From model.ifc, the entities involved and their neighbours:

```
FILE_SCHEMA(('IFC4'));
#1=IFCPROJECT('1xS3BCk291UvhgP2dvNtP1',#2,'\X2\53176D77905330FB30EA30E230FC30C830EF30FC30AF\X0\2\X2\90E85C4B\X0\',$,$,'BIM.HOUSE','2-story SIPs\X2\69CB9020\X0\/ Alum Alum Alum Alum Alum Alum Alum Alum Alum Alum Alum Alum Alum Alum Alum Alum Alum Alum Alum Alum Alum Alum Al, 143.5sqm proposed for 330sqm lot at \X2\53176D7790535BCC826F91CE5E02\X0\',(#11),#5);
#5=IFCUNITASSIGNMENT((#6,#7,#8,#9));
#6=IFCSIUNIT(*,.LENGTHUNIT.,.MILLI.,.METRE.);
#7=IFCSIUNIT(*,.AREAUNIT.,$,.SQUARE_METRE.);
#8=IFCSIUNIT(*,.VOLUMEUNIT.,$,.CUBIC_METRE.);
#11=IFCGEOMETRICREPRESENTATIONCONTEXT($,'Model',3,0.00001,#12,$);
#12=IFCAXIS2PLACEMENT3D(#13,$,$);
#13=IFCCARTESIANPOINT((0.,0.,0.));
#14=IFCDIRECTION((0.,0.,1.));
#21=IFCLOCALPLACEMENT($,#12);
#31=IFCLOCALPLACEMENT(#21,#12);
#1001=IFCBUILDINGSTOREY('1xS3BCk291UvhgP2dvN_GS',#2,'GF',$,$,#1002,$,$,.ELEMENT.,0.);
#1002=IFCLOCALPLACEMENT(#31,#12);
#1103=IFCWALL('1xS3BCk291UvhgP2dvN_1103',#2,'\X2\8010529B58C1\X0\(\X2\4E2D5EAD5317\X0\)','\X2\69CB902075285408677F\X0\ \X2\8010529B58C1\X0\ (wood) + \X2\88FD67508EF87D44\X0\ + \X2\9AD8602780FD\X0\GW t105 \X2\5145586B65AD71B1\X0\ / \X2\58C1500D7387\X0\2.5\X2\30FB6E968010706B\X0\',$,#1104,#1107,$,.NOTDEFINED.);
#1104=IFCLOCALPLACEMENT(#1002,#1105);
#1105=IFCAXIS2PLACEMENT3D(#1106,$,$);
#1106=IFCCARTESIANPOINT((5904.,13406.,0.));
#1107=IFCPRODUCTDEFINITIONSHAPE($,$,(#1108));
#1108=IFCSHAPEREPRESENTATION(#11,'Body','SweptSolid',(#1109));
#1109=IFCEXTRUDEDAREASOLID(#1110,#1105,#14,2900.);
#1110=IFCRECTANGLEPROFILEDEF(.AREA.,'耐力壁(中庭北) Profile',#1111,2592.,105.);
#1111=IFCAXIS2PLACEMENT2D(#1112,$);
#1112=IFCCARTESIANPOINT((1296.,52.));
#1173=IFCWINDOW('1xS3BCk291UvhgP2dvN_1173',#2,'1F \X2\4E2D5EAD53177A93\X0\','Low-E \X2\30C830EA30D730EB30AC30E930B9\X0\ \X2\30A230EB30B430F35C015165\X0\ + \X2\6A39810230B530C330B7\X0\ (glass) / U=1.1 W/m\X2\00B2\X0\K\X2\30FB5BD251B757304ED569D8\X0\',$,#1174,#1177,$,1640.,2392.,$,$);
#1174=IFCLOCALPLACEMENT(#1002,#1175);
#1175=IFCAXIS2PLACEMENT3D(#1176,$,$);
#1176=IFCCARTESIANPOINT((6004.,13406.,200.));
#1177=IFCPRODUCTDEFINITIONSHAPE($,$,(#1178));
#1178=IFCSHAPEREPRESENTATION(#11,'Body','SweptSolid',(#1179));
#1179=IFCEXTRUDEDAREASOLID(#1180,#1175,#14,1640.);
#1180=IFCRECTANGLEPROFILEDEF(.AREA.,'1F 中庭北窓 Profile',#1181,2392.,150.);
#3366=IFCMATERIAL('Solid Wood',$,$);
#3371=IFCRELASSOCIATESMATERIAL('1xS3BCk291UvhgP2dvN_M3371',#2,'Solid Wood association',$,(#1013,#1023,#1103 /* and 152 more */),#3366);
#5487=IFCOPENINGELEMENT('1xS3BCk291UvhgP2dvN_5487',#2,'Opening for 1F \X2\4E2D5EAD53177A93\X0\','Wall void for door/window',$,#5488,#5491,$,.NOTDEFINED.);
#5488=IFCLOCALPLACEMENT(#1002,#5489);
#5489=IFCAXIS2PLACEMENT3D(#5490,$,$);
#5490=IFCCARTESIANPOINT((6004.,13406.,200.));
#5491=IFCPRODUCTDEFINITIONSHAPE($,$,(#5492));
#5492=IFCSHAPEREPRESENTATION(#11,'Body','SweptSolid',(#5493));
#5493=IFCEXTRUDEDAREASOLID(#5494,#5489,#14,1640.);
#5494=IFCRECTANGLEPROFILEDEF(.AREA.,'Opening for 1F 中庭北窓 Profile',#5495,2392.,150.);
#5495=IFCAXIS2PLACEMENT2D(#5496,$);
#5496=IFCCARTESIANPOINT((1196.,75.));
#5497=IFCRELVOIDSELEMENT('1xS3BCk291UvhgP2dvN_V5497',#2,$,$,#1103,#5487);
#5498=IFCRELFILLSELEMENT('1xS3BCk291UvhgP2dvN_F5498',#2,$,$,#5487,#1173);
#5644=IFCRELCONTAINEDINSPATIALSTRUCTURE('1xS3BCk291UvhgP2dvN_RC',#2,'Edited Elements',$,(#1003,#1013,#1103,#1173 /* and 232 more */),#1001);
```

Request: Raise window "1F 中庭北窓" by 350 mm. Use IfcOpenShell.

```python
import numpy as np
import ifcopenshell
import ifcopenshell.api.geometry
import ifcopenshell.util.placement
import ifcopenshell.util.unit

model = ifcopenshell.open("model.ifc")
unit_scale = ifcopenshell.util.unit.calculate_unit_scale(model)

window = model.by_guid("1xS3BCk291UvhgP2dvN_1173")
opening = window.FillsVoids[0].RelatingOpeningElement
dz = 0.35 / unit_scale

shift = np.array([0.0, 0.0, dz])
# The window is not placed relative to its opening, so move both.
for product in (opening, window):
    matrix = ifcopenshell.util.placement.get_local_placement(product.ObjectPlacement)
    matrix[:3, 3] += shift
    ifcopenshell.api.geometry.edit_object_placement(model, product=product, matrix=matrix, is_si=False)

print(f"moved by {dz * unit_scale:+.3f} m")

model.write("model_edited.ifc")
```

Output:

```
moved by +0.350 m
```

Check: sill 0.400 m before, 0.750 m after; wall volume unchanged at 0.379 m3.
